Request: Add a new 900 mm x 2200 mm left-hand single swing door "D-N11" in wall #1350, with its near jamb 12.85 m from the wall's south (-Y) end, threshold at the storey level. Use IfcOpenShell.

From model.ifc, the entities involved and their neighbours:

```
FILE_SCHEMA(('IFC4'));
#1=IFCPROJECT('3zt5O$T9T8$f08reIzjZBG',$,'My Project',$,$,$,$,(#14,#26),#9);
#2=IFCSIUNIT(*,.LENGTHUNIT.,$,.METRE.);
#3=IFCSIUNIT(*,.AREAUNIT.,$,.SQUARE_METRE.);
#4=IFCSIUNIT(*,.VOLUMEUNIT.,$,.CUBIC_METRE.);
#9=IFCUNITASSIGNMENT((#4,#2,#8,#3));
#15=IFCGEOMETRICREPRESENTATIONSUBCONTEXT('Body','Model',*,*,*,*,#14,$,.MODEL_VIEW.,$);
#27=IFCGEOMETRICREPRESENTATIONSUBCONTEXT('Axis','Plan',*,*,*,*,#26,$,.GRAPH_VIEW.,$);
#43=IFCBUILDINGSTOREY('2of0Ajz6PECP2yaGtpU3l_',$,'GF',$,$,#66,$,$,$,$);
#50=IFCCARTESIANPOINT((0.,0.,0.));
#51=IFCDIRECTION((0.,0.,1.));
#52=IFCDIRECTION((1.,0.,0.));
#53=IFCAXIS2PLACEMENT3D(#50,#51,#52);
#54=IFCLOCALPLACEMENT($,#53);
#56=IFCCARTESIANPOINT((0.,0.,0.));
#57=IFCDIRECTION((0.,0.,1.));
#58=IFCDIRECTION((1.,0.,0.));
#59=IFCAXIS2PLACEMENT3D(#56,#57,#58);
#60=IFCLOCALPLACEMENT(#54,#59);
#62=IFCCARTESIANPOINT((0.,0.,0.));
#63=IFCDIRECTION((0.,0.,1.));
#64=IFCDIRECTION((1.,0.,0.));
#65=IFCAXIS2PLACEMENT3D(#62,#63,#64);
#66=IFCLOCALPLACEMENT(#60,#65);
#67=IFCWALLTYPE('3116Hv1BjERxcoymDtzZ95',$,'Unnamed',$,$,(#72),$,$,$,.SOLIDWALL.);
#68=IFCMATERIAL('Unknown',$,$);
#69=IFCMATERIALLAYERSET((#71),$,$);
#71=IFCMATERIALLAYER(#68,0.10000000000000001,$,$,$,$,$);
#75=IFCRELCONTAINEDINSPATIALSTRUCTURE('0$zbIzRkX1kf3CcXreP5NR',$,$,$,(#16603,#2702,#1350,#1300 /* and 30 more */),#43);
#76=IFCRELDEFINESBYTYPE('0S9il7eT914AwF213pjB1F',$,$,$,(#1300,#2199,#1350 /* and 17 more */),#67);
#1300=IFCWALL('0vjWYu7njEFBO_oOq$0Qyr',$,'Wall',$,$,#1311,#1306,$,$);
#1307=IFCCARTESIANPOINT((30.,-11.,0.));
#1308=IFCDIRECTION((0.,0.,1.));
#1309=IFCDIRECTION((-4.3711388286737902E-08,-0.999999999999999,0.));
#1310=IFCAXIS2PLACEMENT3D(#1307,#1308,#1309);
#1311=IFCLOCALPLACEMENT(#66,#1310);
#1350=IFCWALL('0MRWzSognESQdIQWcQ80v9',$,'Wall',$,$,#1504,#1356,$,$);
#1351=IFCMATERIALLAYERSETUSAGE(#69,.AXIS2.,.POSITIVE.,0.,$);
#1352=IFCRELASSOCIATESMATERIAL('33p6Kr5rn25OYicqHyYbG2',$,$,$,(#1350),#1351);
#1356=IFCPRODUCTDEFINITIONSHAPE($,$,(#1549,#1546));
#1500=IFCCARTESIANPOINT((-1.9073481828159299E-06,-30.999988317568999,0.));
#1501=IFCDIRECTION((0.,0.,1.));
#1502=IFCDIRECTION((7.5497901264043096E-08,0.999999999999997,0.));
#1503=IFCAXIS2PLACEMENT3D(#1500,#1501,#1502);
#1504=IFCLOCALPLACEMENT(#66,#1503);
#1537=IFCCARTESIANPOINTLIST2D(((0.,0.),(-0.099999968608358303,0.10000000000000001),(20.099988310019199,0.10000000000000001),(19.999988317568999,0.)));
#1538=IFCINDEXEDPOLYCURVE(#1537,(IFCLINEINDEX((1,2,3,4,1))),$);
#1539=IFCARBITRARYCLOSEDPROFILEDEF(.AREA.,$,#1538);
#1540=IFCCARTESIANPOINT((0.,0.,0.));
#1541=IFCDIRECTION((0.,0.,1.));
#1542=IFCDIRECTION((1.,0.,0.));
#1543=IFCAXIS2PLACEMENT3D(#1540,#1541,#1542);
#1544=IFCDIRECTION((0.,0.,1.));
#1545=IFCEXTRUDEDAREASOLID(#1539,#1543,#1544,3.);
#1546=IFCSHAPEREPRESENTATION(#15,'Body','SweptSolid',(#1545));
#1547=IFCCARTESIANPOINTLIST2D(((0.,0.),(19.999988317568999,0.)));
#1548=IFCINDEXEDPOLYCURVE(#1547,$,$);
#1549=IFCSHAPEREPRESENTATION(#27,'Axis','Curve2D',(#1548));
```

```python
import numpy as np
import ifcopenshell
import ifcopenshell.api.feature
import ifcopenshell.api.geometry
import ifcopenshell.api.root
import ifcopenshell.api.spatial
import ifcopenshell.geom
import ifcopenshell.util.element
import ifcopenshell.util.placement
import ifcopenshell.util.representation
import ifcopenshell.util.shape
import ifcopenshell.util.unit

model = ifcopenshell.open("model.ifc")
unit_scale = ifcopenshell.util.unit.calculate_unit_scale(model)
settings = ifcopenshell.geom.settings()


def volume(element):
    """Net volume in cubic metres, openings subtracted."""
    shape = ifcopenshell.geom.create_shape(settings, element)
    return ifcopenshell.util.shape.get_volume(shape.geometry)


wall = model.by_guid("0MRWzSognESQdIQWcQ80v9")
storey = ifcopenshell.util.element.get_container(wall, ifc_class="IfcBuildingStorey")
context = ifcopenshell.util.representation.get_context(model, "Model", "Body", "MODEL_VIEW")
before = volume(wall)

width, height, from_end, sill = 0.9, 2.2, 12.85, 0.0  # metres

# The wall runs along its own X axis, and the end named is its -X end.
wall_shape = ifcopenshell.geom.create_shape(settings, wall)
x, y, z = ifcopenshell.util.shape.get_vertices(wall_shape.geometry).T
start = x.min() + from_end
face, thickness = float(y.min()), float(y.max() - y.min())
wall_matrix = ifcopenshell.util.placement.get_local_placement(wall.ObjectPlacement)
level = ifcopenshell.util.placement.get_local_placement(storey.ObjectPlacement)[2, 3]


def in_wall(x, y):
    """Placement at x, y metres in the wall's axes, at sill height."""
    matrix = wall_matrix.copy()
    matrix[:, 3] = wall_matrix @ np.array([x / unit_scale, y / unit_scale, 0.0, 1.0])
    matrix[2, 3] = level + sill / unit_scale
    return matrix


# Opening: a box that overshoots both wall faces by 50 mm.
opening = ifcopenshell.api.root.create_entity(model, ifc_class="IfcOpeningElement", predefined_type="OPENING")
box = ifcopenshell.api.geometry.add_wall_representation(
    model, context=context, length=width, height=height, thickness=thickness + 0.1
)
ifcopenshell.api.geometry.assign_representation(model, product=opening, representation=box)
ifcopenshell.api.geometry.edit_object_placement(model, product=opening, matrix=in_wall(start, face - 0.05), is_si=False)
ifcopenshell.api.feature.add_feature(model, feature=opening, element=wall)

door = ifcopenshell.api.root.create_entity(model, ifc_class="IfcDoor", name="D-N11", predefined_type="DOOR")
door.OverallWidth, door.OverallHeight = width / unit_scale, height / unit_scale
door.OperationType = "SINGLE_SWING_LEFT"
body = ifcopenshell.api.geometry.add_door_representation(
    model,
    context=context,
    overall_width=door.OverallWidth,
    overall_height=door.OverallHeight,
    operation_type="SINGLE_SWING_LEFT",
    lining_properties={"LiningDepth": thickness / unit_scale, "ThresholdDepth": thickness / unit_scale},
)
ifcopenshell.api.geometry.assign_representation(model, product=door, representation=body)
ifcopenshell.api.spatial.assign_container(model, products=[door], relating_structure=storey)
ifcopenshell.api.feature.add_filling(model, opening=opening, element=door)

# The lining spans the wall, so the door starts at the wall face.
ifcopenshell.api.geometry.edit_object_placement(model, product=door, matrix=in_wall(start, face), is_si=False)

after = volume(wall)

print(f"wall volume {before:.3f} -> {after:.3f} m3")

model.write("model_rev.ifc")
```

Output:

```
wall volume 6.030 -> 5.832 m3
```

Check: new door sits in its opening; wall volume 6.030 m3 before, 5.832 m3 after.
